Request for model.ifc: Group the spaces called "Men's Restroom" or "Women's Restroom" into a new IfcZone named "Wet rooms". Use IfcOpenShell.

First a look at what the model holds.

```python
import ifcopenshell

model = ifcopenshell.open("model.ifc")
print(model.schema)
seen = {}
for space in model.by_type("IfcSpace"):
    seen[space.LongName] = seen.get(space.LongName, 0) + 1
for name, count in sorted(seen.items(), key=str):
    print(count, "x", name)
print("zones:", [z.Name for z in model.by_type("IfcZone")][:20])
```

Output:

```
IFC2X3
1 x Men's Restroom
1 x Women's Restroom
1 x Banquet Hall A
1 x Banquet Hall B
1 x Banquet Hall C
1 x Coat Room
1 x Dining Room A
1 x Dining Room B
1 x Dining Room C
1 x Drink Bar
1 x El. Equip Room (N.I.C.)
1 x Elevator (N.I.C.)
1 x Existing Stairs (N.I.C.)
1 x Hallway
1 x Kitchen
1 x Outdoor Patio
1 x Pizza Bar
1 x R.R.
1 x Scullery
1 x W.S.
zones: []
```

```python
import ifcopenshell
import ifcopenshell.api.group
import ifcopenshell.api.root

model = ifcopenshell.open("model.ifc")

names = {"Men's Restroom", "Women's Restroom"}
spaces = [s for s in model.by_type("IfcSpace") if s.LongName in names]

zone = ifcopenshell.api.root.create_entity(model, ifc_class="IfcZone", name="Wet rooms")
ifcopenshell.api.group.assign_group(model, products=spaces, group=zone)
print(len(spaces), "spaces in", zone.Name)

model.write("model_edited.ifc")
```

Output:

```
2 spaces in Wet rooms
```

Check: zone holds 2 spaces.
